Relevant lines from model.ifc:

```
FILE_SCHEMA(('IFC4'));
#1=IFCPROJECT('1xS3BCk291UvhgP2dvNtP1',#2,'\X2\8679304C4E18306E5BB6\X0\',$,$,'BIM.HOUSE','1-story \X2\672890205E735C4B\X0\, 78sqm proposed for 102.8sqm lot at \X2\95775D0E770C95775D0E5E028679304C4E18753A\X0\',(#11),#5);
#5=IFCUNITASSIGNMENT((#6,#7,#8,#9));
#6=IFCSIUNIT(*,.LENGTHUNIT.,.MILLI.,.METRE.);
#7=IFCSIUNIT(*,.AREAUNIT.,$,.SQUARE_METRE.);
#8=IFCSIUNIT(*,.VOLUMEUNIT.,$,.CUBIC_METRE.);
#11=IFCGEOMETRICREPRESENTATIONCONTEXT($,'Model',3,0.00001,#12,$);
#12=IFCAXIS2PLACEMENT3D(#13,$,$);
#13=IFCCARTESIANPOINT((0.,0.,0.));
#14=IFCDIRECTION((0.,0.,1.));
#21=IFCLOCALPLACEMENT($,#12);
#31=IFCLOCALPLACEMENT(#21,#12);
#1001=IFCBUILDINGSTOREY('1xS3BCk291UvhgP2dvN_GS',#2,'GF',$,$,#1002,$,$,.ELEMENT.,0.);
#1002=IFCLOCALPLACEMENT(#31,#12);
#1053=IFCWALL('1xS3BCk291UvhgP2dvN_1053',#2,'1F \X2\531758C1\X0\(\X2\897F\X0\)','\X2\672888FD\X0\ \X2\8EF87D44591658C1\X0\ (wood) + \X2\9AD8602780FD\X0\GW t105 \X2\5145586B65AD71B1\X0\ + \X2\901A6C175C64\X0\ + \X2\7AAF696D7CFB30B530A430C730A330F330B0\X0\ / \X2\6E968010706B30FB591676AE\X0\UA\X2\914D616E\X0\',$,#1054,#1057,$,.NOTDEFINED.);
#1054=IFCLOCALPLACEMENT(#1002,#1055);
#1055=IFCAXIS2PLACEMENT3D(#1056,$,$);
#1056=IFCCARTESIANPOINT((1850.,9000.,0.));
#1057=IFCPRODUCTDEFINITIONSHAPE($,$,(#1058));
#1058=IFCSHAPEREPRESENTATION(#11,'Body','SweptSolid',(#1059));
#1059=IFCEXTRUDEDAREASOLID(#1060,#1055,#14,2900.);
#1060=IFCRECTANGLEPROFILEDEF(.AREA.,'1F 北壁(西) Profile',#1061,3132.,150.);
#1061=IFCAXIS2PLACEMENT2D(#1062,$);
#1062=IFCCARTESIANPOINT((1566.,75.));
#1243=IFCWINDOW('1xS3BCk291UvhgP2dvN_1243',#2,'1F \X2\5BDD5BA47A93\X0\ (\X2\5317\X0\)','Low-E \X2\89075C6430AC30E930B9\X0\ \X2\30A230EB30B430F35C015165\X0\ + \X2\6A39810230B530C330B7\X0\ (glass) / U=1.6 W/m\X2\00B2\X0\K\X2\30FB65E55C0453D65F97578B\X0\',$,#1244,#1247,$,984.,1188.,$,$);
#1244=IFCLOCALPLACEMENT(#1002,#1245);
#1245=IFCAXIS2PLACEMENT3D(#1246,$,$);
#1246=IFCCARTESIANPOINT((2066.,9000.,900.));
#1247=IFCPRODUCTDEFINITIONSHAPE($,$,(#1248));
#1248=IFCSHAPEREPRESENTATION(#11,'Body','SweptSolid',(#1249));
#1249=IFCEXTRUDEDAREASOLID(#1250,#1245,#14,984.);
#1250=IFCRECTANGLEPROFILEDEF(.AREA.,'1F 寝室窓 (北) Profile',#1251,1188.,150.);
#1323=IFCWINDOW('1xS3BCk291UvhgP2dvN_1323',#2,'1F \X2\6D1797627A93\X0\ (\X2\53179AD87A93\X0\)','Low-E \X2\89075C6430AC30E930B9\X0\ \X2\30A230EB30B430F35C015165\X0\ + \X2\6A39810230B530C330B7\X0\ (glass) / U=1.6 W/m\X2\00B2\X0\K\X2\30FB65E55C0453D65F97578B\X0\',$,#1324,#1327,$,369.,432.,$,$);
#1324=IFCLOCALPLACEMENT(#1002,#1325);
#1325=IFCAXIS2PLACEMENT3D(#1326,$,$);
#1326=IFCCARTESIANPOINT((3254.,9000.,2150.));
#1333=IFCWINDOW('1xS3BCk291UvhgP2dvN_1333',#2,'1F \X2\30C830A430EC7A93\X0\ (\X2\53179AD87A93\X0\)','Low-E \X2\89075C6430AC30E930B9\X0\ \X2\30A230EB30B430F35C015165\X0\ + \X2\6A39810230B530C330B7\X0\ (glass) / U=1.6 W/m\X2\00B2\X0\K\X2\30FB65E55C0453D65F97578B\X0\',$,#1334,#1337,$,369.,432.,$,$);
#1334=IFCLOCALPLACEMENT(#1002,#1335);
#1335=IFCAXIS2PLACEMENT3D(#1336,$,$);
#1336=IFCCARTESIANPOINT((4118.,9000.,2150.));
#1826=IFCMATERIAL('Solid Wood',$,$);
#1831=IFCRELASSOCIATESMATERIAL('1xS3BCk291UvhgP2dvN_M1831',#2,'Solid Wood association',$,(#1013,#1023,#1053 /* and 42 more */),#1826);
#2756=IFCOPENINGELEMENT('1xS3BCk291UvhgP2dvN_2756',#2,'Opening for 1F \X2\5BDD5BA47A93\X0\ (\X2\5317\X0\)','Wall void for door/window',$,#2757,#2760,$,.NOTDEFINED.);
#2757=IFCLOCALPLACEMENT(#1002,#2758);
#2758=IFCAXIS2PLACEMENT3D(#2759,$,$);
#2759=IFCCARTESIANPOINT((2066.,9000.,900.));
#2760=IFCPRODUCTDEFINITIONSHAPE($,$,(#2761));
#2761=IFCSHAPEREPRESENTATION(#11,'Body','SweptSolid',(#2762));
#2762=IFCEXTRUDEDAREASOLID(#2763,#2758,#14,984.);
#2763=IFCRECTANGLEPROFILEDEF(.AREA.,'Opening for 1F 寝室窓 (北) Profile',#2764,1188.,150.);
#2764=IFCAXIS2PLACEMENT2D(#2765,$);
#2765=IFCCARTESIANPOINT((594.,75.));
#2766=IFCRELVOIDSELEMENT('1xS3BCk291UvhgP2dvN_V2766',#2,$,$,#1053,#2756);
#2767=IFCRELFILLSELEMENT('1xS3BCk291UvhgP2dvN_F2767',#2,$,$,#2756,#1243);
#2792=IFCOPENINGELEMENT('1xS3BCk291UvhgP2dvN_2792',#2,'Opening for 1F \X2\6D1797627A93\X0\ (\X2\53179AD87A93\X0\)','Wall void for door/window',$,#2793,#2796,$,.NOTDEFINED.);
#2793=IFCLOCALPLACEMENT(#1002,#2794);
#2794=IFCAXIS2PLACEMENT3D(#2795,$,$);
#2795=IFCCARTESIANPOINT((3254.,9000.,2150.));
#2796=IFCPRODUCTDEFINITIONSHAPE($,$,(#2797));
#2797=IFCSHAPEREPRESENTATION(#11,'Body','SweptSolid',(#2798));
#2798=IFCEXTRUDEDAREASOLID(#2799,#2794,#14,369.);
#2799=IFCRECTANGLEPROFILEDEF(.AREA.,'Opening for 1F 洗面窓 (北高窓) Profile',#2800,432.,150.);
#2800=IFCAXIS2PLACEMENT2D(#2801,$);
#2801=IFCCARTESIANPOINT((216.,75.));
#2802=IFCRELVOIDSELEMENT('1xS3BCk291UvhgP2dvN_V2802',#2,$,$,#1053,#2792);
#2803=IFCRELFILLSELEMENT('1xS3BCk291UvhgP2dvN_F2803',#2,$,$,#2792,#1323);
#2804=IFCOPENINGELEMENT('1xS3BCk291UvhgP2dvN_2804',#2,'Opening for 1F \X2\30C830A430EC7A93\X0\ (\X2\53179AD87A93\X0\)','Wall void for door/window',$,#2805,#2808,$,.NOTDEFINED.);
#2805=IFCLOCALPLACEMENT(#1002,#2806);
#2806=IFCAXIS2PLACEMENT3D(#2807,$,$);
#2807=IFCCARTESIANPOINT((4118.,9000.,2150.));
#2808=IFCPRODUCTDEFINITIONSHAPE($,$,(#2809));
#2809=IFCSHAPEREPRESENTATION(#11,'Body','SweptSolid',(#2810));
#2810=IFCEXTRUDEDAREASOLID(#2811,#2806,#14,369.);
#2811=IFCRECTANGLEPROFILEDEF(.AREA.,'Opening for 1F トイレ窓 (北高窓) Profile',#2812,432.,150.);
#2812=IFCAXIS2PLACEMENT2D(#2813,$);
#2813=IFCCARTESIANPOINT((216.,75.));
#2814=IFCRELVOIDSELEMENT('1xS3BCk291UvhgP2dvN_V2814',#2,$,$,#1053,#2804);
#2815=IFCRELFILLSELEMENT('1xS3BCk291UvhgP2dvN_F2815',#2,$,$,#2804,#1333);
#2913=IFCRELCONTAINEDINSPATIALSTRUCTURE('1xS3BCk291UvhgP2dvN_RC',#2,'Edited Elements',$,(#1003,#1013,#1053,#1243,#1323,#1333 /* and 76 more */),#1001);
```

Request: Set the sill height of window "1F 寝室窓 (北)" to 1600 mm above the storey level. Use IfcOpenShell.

```python
import numpy as np
import ifcopenshell
import ifcopenshell.api.geometry
import ifcopenshell.geom
import ifcopenshell.util.element
import ifcopenshell.util.placement
import ifcopenshell.util.shape
import ifcopenshell.util.unit

model = ifcopenshell.open("model.ifc")
unit_scale = ifcopenshell.util.unit.calculate_unit_scale(model)

window = model.by_guid("1xS3BCk291UvhgP2dvN_1243")
opening = window.FillsVoids[0].RelatingOpeningElement
storey = ifcopenshell.util.element.get_container(window, ifc_class="IfcBuildingStorey")
level = ifcopenshell.util.placement.get_local_placement(storey.ObjectPlacement)[2, 3]

# The opening's origin need not be at the sill, so measure its lowest point.
shape = ifcopenshell.geom.create_shape(ifcopenshell.geom.settings(), opening)
bottom = ifcopenshell.util.shape.get_shape_bottom_elevation(shape, shape.geometry) / unit_scale
dz = level + 1.6 / unit_scale - bottom

shift = np.array([0.0, 0.0, dz])
# The window is not placed relative to its opening, so move both.
for product in (opening, window):
    matrix = ifcopenshell.util.placement.get_local_placement(product.ObjectPlacement)
    matrix[:3, 3] += shift
    ifcopenshell.api.geometry.edit_object_placement(model, product=product, matrix=matrix, is_si=False)

print(f"moved by {dz * unit_scale:+.3f} m")

model.write("model_edited.ifc")
```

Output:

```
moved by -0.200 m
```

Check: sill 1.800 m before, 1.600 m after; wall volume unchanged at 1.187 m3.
